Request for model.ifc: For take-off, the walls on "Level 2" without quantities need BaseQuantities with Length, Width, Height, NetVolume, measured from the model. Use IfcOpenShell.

First a look at what the model holds.

```python
import ifcopenshell
import ifcopenshell.util.element
import ifcopenshell.util.unit

model = ifcopenshell.open("model.ifc")
print(model.schema)
for unit_type in ("LENGTHUNIT", "AREAUNIT", "VOLUMEUNIT"):
    print(unit_type, ifcopenshell.util.unit.calculate_unit_scale(model, unit_type))
storey = next(s for s in model.by_type("IfcBuildingStorey") if s.Name == "Level 2")
walls = [e for e in ifcopenshell.util.element.get_decomposition(storey) if e.is_a("IfcWall")]
for e in sorted(walls, key=lambda e: e.id()):
    print(e.id(), e.is_a(), e.Name, list(ifcopenshell.util.element.get_psets(e, qtos_only=True)), sep=" | ")
```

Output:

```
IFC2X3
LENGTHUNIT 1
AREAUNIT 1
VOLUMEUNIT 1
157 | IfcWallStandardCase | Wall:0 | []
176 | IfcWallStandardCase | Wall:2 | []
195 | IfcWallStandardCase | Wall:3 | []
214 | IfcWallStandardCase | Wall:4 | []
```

```python
import ifcopenshell
import ifcopenshell.api.pset
import ifcopenshell.geom
import ifcopenshell.util.element
import ifcopenshell.util.shape
import ifcopenshell.util.unit

model = ifcopenshell.open("model.ifc")
unit_scale = ifcopenshell.util.unit.calculate_unit_scale(model)
volume_scale = ifcopenshell.util.unit.calculate_unit_scale(model, "VOLUMEUNIT")
settings = ifcopenshell.geom.settings()

storey = next(s for s in model.by_type("IfcBuildingStorey") if s.Name == "Level 2")
walls = [e for e in ifcopenshell.util.element.get_decomposition(storey) if e.is_a("IfcWall")]

for e in sorted(walls, key=lambda e: e.id()):
    if ifcopenshell.util.element.get_psets(e, qtos_only=True, should_inherit=False):
        continue
    # Geometry comes back in metres, in the element's own axes.
    shape = ifcopenshell.geom.create_shape(settings, e)
    values = {
        "Length": ifcopenshell.util.shape.get_x(shape.geometry) / unit_scale,
        "Width": ifcopenshell.util.shape.get_y(shape.geometry) / unit_scale,
        "Height": ifcopenshell.util.shape.get_z(shape.geometry) / unit_scale,
        "NetVolume": ifcopenshell.util.shape.get_volume(shape.geometry) / volume_scale,
    }
    qto = ifcopenshell.api.pset.add_qto(model, product=e, name="BaseQuantities")
    ifcopenshell.api.pset.edit_qto(model, qto=qto, properties=values)
    print(e.id(), {k: round(v, 3) for k, v in values.items()})

model.write("model_edited.ifc")
```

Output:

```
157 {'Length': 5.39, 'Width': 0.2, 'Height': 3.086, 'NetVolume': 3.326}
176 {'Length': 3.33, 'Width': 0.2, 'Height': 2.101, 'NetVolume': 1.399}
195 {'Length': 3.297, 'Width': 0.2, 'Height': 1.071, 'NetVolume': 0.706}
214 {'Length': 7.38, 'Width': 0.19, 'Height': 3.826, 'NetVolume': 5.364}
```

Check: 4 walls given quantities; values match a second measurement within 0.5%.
